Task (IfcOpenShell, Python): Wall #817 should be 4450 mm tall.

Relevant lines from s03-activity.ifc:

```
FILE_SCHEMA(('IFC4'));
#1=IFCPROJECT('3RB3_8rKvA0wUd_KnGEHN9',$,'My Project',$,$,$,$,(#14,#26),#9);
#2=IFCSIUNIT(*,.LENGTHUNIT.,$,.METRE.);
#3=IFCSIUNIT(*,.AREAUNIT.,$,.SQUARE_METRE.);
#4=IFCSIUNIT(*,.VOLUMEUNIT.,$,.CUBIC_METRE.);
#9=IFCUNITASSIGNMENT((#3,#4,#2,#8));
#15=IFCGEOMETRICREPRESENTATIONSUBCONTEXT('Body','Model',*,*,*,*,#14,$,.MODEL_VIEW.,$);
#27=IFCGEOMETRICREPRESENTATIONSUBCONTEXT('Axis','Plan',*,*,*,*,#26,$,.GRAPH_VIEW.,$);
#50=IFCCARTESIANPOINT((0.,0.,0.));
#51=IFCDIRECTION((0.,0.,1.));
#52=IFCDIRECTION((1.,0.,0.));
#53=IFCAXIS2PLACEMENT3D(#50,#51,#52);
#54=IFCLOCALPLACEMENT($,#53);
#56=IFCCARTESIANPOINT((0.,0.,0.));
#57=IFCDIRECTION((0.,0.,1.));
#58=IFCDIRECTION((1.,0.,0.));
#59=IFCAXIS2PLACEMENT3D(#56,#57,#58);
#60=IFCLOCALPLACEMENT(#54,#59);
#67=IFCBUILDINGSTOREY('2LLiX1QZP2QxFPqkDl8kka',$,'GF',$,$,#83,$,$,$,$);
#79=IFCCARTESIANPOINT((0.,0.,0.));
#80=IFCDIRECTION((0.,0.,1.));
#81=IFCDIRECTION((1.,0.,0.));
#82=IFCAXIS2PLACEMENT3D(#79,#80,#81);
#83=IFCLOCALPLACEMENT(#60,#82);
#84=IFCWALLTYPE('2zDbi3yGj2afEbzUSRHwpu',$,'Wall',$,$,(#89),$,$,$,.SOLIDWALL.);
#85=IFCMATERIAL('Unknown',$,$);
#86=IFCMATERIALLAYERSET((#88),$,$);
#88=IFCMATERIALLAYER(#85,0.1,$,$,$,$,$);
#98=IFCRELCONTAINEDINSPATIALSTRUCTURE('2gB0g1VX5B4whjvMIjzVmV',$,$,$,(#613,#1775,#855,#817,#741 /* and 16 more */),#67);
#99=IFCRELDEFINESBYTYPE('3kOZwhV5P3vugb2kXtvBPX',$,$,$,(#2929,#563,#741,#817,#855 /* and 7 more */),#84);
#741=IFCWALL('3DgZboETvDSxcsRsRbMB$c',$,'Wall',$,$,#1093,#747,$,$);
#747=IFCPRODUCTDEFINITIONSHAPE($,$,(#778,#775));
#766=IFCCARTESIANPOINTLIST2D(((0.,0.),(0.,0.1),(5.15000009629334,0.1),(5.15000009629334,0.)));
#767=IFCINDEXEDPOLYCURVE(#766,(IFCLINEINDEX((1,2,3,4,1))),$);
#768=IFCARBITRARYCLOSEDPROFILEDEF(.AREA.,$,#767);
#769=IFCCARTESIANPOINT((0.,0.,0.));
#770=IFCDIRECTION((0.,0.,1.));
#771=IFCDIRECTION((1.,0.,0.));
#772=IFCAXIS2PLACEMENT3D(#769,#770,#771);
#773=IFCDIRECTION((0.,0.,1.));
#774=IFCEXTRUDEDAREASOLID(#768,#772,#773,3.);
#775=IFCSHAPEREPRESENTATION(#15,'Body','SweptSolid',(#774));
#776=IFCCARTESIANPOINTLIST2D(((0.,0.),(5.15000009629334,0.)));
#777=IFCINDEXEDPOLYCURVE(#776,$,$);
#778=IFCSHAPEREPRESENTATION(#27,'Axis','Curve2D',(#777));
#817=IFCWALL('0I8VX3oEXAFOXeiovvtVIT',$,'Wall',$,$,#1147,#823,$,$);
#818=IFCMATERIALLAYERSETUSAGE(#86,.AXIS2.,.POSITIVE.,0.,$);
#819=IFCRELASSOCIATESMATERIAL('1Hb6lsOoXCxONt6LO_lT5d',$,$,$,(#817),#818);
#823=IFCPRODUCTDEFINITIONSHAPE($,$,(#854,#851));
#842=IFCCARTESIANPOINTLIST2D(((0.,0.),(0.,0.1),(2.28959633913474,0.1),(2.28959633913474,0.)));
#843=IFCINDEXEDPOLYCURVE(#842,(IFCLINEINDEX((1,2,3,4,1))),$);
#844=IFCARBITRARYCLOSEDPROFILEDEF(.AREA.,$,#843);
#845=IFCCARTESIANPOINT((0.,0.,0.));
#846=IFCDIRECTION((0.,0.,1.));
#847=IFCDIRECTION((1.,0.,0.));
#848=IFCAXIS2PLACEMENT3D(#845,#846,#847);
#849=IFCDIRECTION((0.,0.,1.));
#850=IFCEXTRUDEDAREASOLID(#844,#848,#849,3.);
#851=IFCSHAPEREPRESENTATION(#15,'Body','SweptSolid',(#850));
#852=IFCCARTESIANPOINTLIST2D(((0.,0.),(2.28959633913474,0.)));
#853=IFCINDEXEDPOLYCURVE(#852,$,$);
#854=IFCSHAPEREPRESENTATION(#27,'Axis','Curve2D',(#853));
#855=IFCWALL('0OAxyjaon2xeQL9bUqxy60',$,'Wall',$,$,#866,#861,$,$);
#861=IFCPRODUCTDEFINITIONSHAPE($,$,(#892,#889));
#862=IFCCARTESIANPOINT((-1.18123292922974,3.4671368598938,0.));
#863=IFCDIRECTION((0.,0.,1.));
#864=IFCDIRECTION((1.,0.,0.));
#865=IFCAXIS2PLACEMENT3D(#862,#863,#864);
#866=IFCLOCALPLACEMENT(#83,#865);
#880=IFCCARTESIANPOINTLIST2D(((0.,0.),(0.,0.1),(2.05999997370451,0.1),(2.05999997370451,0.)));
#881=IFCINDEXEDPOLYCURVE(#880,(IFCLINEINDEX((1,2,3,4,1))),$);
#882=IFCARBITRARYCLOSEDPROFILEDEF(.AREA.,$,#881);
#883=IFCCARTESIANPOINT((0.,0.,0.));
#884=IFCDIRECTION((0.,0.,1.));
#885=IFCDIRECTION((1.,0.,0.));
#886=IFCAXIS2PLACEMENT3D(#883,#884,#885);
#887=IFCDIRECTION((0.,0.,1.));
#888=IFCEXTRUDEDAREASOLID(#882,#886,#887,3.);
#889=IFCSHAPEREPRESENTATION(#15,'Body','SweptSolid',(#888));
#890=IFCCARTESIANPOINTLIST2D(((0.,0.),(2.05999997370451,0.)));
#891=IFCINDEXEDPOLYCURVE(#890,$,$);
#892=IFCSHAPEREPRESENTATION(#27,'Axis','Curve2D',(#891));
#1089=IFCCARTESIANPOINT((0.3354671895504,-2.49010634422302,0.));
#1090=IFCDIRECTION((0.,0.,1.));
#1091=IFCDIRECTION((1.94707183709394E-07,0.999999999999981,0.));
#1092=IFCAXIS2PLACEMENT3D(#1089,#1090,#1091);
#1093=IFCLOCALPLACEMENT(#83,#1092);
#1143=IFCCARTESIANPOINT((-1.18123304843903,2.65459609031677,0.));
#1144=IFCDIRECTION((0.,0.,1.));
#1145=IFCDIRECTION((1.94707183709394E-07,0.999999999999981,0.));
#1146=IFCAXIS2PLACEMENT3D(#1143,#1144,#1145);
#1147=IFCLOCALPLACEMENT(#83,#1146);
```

```python
import ifcopenshell
import ifcopenshell.geom
import ifcopenshell.util.representation
import ifcopenshell.util.shape
import ifcopenshell.util.unit

model = ifcopenshell.open("s03-activity.ifc")
unit_scale = ifcopenshell.util.unit.calculate_unit_scale(model)
settings = ifcopenshell.geom.settings()


def volume(element):
    """Net volume in cubic metres, openings subtracted."""
    shape = ifcopenshell.geom.create_shape(settings, element)
    return ifcopenshell.util.shape.get_volume(shape.geometry)


wall = model.by_id(817)
before = volume(wall)

body = ifcopenshell.util.representation.get_representation(wall, "Model", "Body")
solid = body.Items[0]
old_height = solid.Depth
solid.Depth = 4.45 / unit_scale
after = volume(wall)

print(f"height {old_height:g} -> {solid.Depth:g}, volume {before:.3f} -> {after:.3f} m3")

model.write("s03-activity_edited.ifc")
```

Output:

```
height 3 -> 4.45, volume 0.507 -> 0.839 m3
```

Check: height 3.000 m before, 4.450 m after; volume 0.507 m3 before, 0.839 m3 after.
